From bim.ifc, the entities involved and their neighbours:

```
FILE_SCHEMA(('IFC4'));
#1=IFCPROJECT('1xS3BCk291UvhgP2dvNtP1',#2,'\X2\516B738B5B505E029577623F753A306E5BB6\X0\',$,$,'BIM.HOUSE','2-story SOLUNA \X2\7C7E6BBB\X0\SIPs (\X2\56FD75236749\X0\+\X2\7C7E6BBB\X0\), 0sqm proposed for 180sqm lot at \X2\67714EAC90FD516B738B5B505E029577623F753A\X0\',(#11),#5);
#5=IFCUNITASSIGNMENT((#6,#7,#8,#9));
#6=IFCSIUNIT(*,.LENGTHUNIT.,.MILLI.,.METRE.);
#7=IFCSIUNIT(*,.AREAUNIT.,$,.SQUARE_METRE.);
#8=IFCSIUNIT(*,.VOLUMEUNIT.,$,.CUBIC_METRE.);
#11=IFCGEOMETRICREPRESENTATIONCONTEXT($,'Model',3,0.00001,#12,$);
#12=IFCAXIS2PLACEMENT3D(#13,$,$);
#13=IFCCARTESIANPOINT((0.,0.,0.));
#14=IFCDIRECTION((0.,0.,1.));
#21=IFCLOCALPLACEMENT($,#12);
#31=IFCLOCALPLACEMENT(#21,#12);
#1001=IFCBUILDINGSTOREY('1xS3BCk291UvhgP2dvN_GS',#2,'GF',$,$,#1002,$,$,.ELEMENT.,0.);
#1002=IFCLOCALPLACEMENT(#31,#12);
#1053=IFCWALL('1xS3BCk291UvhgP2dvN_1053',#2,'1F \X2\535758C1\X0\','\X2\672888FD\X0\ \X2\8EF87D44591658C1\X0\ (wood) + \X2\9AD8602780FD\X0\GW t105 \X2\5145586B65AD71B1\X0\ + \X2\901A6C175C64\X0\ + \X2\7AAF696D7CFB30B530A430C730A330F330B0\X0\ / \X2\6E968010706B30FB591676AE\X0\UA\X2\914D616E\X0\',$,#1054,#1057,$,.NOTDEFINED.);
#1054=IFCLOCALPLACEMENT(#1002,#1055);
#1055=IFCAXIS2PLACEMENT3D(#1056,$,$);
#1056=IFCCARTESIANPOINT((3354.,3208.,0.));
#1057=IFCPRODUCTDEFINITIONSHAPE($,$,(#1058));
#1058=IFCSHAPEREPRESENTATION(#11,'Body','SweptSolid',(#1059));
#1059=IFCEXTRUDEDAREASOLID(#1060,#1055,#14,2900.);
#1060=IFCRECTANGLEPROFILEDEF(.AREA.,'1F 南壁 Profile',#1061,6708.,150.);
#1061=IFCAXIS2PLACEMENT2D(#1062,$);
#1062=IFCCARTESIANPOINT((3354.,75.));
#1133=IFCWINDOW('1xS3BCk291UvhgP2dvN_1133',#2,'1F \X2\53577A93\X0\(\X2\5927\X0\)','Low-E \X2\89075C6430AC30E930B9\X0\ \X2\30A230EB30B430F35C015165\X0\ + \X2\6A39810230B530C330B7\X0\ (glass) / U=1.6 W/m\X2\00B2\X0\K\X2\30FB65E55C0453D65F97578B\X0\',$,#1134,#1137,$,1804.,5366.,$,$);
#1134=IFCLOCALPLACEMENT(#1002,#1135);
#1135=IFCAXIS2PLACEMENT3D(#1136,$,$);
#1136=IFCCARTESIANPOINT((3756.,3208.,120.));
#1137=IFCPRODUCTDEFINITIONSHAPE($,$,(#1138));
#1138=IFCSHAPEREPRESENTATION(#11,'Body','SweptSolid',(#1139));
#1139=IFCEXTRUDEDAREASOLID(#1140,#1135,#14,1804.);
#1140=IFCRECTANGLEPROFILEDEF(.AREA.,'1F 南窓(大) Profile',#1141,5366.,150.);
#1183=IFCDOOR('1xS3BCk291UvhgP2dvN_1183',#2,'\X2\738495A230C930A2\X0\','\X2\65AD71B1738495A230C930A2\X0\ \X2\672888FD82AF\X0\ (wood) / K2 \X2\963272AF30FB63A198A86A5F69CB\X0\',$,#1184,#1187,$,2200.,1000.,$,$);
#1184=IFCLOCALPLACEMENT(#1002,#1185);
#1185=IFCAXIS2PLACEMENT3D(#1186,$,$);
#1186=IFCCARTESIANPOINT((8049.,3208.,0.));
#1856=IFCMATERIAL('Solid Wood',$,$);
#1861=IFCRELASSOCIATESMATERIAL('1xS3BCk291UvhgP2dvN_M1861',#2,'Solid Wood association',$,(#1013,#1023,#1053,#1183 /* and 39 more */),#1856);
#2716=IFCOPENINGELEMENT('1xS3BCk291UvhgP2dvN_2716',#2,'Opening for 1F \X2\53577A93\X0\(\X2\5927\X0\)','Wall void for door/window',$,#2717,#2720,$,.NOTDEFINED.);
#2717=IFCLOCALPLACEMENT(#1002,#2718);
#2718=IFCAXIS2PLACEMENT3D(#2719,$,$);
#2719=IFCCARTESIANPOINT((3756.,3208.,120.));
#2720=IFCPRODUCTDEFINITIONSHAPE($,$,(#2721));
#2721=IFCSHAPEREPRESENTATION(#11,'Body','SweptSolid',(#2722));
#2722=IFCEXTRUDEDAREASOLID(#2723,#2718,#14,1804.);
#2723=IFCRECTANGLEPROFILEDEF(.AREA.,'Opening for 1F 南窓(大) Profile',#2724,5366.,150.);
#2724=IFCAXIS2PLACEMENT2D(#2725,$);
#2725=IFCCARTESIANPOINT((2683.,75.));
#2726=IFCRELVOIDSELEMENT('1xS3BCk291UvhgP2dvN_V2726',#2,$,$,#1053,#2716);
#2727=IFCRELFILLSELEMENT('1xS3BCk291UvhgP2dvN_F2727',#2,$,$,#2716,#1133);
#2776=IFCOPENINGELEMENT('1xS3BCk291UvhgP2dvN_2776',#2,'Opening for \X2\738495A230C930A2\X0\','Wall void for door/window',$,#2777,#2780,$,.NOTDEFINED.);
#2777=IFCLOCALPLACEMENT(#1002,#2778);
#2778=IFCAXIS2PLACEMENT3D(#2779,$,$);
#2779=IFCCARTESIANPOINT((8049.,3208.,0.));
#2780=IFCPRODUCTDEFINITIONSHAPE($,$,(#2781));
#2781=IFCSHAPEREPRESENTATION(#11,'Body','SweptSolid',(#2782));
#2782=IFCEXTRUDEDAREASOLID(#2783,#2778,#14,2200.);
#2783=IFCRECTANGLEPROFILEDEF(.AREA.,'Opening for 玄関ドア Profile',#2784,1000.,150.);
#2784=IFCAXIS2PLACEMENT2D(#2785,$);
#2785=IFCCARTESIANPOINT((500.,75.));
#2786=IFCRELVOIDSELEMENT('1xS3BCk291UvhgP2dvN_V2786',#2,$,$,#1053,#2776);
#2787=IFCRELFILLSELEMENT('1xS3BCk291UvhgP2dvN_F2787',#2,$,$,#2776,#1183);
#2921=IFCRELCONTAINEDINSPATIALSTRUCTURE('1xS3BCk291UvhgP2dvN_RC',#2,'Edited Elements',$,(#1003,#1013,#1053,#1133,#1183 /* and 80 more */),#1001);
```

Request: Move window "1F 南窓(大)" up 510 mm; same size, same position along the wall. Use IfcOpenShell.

```python
import numpy as np
import ifcopenshell
import ifcopenshell.api.geometry
import ifcopenshell.util.placement
import ifcopenshell.util.unit

model = ifcopenshell.open("bim.ifc")
unit_scale = ifcopenshell.util.unit.calculate_unit_scale(model)

window = model.by_guid("1xS3BCk291UvhgP2dvN_1133")
opening = window.FillsVoids[0].RelatingOpeningElement
dz = 0.51 / unit_scale

shift = np.array([0.0, 0.0, dz])
# The window is not placed relative to its opening, so move both.
for product in (opening, window):
    matrix = ifcopenshell.util.placement.get_local_placement(product.ObjectPlacement)
    matrix[:3, 3] += shift
    ifcopenshell.api.geometry.edit_object_placement(model, product=product, matrix=matrix, is_si=False)

print(f"moved by {dz * unit_scale:+.3f} m")

model.write("bim_rev.ifc")
```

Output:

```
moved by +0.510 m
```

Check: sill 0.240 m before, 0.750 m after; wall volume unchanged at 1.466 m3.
